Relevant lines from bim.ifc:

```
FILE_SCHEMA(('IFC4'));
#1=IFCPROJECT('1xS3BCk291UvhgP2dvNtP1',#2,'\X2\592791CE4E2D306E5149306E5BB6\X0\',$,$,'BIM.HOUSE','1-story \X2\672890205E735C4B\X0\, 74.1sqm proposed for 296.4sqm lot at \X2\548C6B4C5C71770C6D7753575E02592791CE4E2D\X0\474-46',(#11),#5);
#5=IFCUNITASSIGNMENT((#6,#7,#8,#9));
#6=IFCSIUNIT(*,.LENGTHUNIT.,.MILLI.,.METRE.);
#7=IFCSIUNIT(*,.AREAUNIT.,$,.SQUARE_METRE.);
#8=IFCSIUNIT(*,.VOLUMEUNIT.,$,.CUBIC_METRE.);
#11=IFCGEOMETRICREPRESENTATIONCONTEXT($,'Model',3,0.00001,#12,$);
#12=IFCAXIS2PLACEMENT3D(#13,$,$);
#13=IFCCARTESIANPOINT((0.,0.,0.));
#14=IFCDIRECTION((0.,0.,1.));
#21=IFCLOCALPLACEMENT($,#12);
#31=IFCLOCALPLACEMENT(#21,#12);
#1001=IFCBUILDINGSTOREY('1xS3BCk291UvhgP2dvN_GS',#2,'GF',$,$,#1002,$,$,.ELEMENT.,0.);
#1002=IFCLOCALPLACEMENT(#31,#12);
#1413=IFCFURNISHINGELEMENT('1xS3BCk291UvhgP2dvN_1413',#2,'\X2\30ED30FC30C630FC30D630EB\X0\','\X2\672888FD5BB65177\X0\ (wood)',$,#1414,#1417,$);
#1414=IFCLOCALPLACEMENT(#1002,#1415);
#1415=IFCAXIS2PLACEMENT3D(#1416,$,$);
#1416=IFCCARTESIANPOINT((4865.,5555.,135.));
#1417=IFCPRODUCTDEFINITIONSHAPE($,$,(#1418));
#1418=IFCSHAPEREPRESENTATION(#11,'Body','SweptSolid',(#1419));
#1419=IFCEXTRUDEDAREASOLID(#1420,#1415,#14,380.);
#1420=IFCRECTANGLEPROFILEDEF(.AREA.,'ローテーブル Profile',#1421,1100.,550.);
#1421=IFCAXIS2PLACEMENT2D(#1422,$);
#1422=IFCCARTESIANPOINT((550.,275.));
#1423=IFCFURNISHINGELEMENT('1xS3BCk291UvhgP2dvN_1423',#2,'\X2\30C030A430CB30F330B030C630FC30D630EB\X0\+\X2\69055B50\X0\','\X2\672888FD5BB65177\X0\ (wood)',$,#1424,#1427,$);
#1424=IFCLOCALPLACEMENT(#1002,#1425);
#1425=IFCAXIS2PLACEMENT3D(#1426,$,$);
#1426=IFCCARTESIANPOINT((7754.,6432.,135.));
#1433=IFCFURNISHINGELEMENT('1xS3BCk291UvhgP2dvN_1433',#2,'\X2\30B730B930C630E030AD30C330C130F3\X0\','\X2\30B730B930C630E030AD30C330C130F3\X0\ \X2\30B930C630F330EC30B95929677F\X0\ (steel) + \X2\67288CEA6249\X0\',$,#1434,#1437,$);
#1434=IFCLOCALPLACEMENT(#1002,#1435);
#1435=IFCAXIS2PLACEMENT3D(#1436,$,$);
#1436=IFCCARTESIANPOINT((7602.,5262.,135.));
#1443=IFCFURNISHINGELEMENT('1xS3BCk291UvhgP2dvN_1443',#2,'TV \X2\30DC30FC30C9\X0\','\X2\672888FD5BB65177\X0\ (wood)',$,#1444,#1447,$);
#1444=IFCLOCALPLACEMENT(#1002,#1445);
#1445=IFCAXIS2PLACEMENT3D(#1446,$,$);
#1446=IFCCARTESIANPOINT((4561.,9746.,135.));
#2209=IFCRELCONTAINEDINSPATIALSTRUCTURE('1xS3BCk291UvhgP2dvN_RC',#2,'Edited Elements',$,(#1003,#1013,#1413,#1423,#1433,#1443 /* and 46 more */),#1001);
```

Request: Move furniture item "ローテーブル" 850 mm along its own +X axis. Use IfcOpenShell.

```python
import ifcopenshell
import ifcopenshell.api.geometry
import ifcopenshell.util.placement
import ifcopenshell.util.unit

model = ifcopenshell.open("bim.ifc")
unit_scale = ifcopenshell.util.unit.calculate_unit_scale(model)

item = model.by_guid("1xS3BCk291UvhgP2dvN_1413")
matrix = ifcopenshell.util.placement.get_local_placement(item.ObjectPlacement)
matrix[:3, 3] += matrix[:3, 0] * 0.85 / unit_scale
ifcopenshell.api.geometry.edit_object_placement(model, product=item, matrix=matrix, is_si=False)

print(ifcopenshell.util.placement.get_local_placement(item.ObjectPlacement).round(3) + 0.0)

model.write("bim_rev.ifc")
```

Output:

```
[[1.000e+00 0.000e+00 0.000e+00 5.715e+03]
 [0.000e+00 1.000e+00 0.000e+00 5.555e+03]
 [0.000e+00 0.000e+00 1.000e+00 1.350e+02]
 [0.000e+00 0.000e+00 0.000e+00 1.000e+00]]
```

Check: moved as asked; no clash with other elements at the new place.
